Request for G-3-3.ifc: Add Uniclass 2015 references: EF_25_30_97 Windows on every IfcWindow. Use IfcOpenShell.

First a look at what the model holds.

```python
import ifcopenshell

model = ifcopenshell.open("G-3-3.ifc")
print(model.schema)
print("classifications:", [c.Name for c in model.by_type("IfcClassification")])
for ifc_class in ("IfcDoor", "IfcRoof", "IfcStair", "IfcWall", "IfcWindow"):
    print(ifc_class, len(model.by_type(ifc_class)))
```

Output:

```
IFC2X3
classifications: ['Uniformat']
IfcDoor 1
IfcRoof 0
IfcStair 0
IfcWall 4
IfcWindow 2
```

```python
import ifcopenshell
import ifcopenshell.api.classification

model = ifcopenshell.open("G-3-3.ifc")

# IFC2X3 requires Source and Edition and has no link from the project to the system.
system = model.create_entity("IfcClassification", Source="NBS", Edition="2015", Name="Uniclass 2015")

codes = {
    "IfcWindow": ("EF_25_30_97", "Windows"),
}
for ifc_class, (code, name) in codes.items():
    products = model.by_type(ifc_class)
    ifcopenshell.api.classification.add_reference(
        model, products=products, classification=system, identification=code, name=name
    )
    print(code, len(products))

model.write("G-3-3-out.ifc")
```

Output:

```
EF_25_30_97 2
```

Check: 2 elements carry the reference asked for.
